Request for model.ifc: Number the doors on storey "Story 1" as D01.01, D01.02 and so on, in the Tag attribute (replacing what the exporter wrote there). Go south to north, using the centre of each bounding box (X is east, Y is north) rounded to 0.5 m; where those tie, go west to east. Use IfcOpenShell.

First a look at what the model holds.

```python
import ifcopenshell
import ifcopenshell.util.element
import ifcopenshell.util.placement

model = ifcopenshell.open("model.ifc")
print(model.schema)
storey = next(s for s in model.by_type("IfcBuildingStorey") if s.Name == "Story 1")
doors = [e for e in ifcopenshell.util.element.get_decomposition(storey) if e.is_a("IfcDoor")]
for e in sorted(doors, key=lambda e: e.id()):
    origin = ifcopenshell.util.placement.get_local_placement(e.ObjectPlacement)[:3, 3]
    print(e.id(), e.Tag, e.Name, origin.round(2) + 0.0, sep=" | ")
```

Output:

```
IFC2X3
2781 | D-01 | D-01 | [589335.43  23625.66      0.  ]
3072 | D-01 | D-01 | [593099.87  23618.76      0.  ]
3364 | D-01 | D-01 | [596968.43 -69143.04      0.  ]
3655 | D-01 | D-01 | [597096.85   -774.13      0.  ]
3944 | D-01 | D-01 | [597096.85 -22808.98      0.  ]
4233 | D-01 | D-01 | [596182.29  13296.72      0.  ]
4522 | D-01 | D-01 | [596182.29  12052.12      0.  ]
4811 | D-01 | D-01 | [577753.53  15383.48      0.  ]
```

```python
import ifcopenshell
import ifcopenshell.geom
import ifcopenshell.util.element
import ifcopenshell.util.shape

model = ifcopenshell.open("model.ifc")
settings = ifcopenshell.geom.settings()
settings.set("use-world-coords", True)


def centre(element):
    shape = ifcopenshell.geom.create_shape(settings, element)
    return ifcopenshell.util.shape.get_bbox_centroid(shape.geometry)


storey = next(s for s in model.by_type("IfcBuildingStorey") if s.Name == "Story 1")
doors = [e for e in ifcopenshell.util.element.get_decomposition(storey) if e.is_a("IfcDoor")]

# Insertion points can sit at a corner or the storey origin, so sort by the geometry (in metres).
centres = {e: centre(e) for e in doors}
doors.sort(key=lambda e: (round(centres[e][1] / 0.5), centres[e][0]))

for i, e in enumerate(doors, start=1):
    number = f"D01.{i:02d}"
    e.Tag = number
    print(e.id(), number)

model.write("model_v2.ifc")
```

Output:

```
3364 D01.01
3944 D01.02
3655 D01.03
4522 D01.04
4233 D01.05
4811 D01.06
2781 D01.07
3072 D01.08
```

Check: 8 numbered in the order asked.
